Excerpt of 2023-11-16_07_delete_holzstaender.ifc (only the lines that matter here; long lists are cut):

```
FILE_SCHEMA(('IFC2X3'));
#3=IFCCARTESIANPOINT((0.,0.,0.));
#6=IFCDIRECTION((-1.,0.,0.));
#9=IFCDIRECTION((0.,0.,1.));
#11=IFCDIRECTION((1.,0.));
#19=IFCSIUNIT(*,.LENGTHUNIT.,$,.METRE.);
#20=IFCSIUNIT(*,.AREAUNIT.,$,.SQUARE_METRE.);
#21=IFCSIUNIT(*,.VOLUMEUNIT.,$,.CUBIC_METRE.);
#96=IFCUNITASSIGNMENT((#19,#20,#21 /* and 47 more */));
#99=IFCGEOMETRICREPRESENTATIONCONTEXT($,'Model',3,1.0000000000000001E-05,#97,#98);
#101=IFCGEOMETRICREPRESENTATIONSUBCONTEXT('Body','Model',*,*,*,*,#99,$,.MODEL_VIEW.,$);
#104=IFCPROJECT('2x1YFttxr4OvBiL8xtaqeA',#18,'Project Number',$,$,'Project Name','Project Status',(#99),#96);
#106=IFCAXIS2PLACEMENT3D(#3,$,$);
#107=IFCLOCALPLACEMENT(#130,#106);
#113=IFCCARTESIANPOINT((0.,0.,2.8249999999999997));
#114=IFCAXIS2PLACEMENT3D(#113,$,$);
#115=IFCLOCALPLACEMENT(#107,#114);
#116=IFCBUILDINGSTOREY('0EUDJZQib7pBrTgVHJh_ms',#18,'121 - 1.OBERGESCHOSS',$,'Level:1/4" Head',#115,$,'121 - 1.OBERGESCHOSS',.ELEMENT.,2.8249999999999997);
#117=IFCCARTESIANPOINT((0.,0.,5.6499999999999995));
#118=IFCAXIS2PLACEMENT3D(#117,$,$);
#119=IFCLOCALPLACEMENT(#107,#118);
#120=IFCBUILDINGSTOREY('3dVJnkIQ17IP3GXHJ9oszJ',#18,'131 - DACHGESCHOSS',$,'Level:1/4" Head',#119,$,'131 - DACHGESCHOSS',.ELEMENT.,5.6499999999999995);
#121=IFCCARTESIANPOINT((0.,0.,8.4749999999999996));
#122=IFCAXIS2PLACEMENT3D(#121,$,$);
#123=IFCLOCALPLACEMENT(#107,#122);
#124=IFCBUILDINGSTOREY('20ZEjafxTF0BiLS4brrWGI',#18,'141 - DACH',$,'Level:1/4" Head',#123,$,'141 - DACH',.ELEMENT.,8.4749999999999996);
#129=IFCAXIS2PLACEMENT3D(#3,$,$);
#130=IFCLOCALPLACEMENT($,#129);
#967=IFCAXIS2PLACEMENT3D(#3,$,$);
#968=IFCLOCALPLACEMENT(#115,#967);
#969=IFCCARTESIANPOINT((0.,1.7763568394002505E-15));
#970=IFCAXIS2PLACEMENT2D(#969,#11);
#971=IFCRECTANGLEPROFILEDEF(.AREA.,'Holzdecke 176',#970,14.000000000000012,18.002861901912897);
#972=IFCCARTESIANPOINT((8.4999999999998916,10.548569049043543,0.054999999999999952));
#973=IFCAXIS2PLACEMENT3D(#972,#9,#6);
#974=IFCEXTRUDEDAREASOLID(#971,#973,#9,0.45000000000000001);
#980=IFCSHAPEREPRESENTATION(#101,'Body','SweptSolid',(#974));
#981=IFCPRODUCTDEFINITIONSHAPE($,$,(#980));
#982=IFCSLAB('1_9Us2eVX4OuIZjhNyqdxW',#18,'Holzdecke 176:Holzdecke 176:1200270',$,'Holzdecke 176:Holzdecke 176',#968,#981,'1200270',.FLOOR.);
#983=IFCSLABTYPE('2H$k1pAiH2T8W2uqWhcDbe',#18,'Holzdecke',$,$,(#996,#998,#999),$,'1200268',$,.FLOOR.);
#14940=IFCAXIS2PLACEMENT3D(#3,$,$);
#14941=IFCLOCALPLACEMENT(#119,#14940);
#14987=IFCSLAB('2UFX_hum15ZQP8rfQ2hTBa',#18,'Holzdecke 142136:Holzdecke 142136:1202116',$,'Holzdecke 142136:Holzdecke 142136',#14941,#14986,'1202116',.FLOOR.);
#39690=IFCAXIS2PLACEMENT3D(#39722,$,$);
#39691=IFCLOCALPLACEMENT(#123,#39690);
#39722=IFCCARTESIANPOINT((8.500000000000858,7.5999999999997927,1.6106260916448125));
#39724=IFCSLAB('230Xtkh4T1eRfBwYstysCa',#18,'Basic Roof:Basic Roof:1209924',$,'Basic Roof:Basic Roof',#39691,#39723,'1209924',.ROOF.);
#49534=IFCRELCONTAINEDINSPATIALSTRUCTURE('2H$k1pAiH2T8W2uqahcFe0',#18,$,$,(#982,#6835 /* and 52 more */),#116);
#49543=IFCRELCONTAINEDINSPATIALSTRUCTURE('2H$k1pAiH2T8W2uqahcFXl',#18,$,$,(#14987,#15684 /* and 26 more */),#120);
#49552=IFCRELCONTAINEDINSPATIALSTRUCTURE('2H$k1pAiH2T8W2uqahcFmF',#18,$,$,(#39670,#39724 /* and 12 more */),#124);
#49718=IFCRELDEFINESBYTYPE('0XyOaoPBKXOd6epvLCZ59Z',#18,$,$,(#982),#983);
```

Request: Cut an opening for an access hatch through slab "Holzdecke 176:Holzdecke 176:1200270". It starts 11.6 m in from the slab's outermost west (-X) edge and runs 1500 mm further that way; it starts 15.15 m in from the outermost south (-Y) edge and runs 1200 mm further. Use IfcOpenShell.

```python
import numpy as np
import ifcopenshell
import ifcopenshell.api.feature
import ifcopenshell.api.geometry
import ifcopenshell.api.root
import ifcopenshell.geom
import ifcopenshell.util.placement
import ifcopenshell.util.representation
import ifcopenshell.util.shape
import ifcopenshell.util.unit

model = ifcopenshell.open("2023-11-16_07_delete_holzstaender.ifc")
unit_scale = ifcopenshell.util.unit.calculate_unit_scale(model)
settings = ifcopenshell.geom.settings()


def volume(element):
    """Net volume in cubic metres, openings subtracted."""
    shape = ifcopenshell.geom.create_shape(settings, element)
    return ifcopenshell.util.shape.get_volume(shape.geometry)


slab = model.by_guid("1_9Us2eVX4OuIZjhNyqdxW")
before = volume(slab)

# Extent in the slab's own axes, in metres. The edges named are its -X and -Y sides.
slab_shape = ifcopenshell.geom.create_shape(settings, slab)
vertices = ifcopenshell.util.shape.get_vertices(slab_shape.geometry)
x_min, y_min, bottom = vertices.min(axis=0)
top = vertices[:, 2].max()

opening = ifcopenshell.api.root.create_entity(model, ifc_class="IfcOpeningElement", name="Access hatch opening")
context = ifcopenshell.util.representation.get_context(model, "Model", "Body", "MODEL_VIEW")
width, depth = 1.5, 1.2
outline = [(0.0, 0.0), (width, 0.0), (width, depth), (0.0, depth), (0.0, 0.0)]
# Overshoot both faces by 50 mm so the cut is clean.
shape = ifcopenshell.api.geometry.add_slab_representation(
    model, context=context, depth=top - bottom + 0.1, polyline=outline
)
ifcopenshell.api.geometry.assign_representation(model, product=opening, representation=shape)

matrix = ifcopenshell.util.placement.get_local_placement(slab.ObjectPlacement)
matrix[:, 3] = matrix @ np.append(np.array([x_min + 11.6, y_min + 15.15, bottom - 0.05]) / unit_scale, 1.0)
ifcopenshell.api.geometry.edit_object_placement(model, product=opening, matrix=matrix, is_si=False)
ifcopenshell.api.feature.add_feature(model, feature=opening, element=slab)

after = volume(slab)

print(f"slab volume {before:.3f} -> {after:.3f} m3")

model.write("2023-11-16_07_delete_holzstaender_v2.ifc")
```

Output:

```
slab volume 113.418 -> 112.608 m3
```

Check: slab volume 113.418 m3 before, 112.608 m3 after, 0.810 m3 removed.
